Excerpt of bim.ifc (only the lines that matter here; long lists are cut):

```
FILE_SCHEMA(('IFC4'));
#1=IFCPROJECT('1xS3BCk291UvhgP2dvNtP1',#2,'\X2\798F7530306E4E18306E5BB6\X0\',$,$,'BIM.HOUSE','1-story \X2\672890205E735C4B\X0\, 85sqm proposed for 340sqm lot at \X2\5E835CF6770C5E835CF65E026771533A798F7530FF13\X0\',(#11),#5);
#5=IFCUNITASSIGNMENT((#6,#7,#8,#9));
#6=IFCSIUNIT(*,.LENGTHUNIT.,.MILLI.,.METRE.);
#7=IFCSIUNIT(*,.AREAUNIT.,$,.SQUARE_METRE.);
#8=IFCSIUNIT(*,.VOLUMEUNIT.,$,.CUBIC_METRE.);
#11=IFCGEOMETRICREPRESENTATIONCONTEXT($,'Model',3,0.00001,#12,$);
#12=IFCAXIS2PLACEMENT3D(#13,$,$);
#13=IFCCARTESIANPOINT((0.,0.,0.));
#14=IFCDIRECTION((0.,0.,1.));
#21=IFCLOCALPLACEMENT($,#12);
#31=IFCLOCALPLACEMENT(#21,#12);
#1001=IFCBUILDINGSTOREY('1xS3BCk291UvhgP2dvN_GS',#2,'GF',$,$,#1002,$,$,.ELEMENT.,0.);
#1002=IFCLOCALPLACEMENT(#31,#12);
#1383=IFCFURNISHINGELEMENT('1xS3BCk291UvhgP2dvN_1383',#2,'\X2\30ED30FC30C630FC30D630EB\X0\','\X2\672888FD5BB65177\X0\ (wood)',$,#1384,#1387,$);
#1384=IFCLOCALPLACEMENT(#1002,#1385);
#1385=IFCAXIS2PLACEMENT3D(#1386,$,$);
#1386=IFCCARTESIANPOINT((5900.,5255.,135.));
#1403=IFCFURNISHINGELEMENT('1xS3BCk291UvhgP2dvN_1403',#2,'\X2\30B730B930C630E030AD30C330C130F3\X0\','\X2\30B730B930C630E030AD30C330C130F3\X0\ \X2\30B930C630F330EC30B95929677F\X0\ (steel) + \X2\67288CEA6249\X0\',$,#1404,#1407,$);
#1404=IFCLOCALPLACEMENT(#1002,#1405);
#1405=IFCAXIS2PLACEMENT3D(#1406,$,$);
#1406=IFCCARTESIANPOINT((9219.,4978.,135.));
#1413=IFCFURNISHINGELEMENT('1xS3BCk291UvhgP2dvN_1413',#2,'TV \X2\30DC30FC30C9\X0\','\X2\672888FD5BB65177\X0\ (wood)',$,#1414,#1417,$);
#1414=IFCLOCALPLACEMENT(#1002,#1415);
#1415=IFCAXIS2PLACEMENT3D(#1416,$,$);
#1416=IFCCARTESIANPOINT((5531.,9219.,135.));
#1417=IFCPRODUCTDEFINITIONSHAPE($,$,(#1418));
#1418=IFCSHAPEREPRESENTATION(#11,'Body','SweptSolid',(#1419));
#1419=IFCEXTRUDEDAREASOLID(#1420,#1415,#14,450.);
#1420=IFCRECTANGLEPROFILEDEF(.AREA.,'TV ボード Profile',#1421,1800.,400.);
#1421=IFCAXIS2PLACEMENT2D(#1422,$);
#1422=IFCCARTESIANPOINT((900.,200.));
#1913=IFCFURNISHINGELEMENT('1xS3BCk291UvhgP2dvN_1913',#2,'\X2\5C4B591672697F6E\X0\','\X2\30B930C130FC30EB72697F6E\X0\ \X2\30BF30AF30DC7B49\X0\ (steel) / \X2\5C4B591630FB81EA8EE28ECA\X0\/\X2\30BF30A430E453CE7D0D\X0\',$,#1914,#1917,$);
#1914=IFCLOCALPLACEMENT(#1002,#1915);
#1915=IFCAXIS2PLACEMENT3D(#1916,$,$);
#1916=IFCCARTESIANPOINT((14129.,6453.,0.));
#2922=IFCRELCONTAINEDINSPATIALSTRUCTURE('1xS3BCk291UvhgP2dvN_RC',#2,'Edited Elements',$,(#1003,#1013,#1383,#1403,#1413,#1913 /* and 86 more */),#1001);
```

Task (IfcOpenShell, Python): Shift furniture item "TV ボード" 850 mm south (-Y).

```python
import ifcopenshell
import ifcopenshell.api.geometry
import ifcopenshell.util.placement
import ifcopenshell.util.unit

model = ifcopenshell.open("bim.ifc")
unit_scale = ifcopenshell.util.unit.calculate_unit_scale(model)

item = model.by_id(1413)
matrix = ifcopenshell.util.placement.get_local_placement(item.ObjectPlacement)
matrix[1, 3] -= 0.85 / unit_scale
ifcopenshell.api.geometry.edit_object_placement(model, product=item, matrix=matrix, is_si=False)

print(ifcopenshell.util.placement.get_local_placement(item.ObjectPlacement).round(3) + 0.0)

model.write("bim_updated.ifc")
```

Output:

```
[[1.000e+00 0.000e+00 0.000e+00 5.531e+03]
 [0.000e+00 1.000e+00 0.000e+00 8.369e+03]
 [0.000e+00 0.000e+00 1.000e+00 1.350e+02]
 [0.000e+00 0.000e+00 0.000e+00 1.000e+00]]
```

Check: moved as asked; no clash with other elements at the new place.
